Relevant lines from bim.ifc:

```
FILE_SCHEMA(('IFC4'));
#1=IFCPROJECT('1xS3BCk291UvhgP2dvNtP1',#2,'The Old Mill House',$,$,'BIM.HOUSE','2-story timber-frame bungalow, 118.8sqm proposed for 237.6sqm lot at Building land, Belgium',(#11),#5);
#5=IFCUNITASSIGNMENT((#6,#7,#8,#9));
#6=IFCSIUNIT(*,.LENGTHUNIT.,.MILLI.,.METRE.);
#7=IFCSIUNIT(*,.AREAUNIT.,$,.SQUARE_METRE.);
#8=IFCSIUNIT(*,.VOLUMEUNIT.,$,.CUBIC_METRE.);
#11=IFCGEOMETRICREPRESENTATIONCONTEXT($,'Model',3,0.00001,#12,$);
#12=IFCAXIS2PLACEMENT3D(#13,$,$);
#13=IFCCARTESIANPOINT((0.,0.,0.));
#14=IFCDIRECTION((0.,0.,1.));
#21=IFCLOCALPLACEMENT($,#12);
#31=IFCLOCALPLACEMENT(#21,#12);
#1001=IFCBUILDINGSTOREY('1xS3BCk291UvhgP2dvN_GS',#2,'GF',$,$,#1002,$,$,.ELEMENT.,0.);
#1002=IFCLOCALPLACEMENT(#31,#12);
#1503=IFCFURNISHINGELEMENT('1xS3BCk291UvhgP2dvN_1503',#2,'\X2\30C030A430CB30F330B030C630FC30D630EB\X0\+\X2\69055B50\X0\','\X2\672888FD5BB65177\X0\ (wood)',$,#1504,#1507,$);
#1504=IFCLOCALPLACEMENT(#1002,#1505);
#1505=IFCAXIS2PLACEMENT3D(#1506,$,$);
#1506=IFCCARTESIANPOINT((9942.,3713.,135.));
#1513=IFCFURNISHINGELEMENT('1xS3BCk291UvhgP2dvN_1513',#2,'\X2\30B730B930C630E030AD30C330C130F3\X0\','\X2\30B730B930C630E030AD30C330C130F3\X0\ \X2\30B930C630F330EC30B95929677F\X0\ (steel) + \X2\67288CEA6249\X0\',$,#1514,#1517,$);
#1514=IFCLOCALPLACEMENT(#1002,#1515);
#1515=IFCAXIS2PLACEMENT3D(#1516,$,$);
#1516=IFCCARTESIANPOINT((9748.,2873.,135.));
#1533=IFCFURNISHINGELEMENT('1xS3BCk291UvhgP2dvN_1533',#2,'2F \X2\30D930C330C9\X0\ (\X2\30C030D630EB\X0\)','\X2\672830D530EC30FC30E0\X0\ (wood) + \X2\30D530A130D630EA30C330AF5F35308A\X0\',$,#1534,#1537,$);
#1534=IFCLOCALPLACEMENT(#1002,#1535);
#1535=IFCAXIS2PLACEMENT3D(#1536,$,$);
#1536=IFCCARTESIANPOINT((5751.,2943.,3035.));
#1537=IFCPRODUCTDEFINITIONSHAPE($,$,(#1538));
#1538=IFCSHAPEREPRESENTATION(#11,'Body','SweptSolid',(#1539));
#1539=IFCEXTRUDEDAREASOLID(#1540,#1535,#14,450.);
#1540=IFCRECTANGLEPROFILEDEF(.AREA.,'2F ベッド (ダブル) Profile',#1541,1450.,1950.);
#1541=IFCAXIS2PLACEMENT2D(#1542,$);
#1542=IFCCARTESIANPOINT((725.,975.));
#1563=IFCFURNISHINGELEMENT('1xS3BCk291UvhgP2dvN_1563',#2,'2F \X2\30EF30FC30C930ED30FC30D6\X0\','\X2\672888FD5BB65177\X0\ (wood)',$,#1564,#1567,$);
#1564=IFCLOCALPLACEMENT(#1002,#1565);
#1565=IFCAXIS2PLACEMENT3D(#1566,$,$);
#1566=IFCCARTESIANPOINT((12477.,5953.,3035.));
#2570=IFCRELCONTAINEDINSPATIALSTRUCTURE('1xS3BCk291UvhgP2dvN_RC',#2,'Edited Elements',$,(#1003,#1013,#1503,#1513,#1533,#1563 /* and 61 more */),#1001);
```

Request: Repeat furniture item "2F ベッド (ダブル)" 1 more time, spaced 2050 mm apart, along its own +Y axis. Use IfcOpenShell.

```python
import ifcopenshell
import ifcopenshell.api.geometry
import ifcopenshell.api.root
import ifcopenshell.util.element
import ifcopenshell.util.placement
import ifcopenshell.util.unit

model = ifcopenshell.open("bim.ifc")
unit_scale = ifcopenshell.util.unit.calculate_unit_scale(model)


def reuse_history(source, copy):
    """copy_class also copies each property set's owner history, people and application; keep the originals."""
    for rel in copy.IsDefinedBy:
        if rel.is_a("IfcRelDefinesByProperties") and (history := rel.RelatingPropertyDefinition.OwnerHistory):
            rel.RelatingPropertyDefinition.OwnerHistory = source.OwnerHistory
            ifcopenshell.util.element.remove_deep2(model, history)


source = model.by_guid("1xS3BCk291UvhgP2dvN_1533")
base = ifcopenshell.util.placement.get_local_placement(source.ObjectPlacement)
step = base[:3, 1] * 2.05 / unit_scale

for i in range(1, 2):
    copy = ifcopenshell.api.root.copy_class(model, product=source)
    copy.Representation = ifcopenshell.util.element.copy_deep(
        model, source.Representation, exclude=["IfcGeometricRepresentationContext", "IfcRepresentationMap"]
    )
    reuse_history(source, copy)
    matrix = base.copy()
    matrix[:3, 3] += i * step
    print("added at", matrix[:3, 3].round(3) + 0.0)
    ifcopenshell.api.geometry.edit_object_placement(model, product=copy, matrix=matrix, is_si=False)

model.write("bim_rev.ifc")
```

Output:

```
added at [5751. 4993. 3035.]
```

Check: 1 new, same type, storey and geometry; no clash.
